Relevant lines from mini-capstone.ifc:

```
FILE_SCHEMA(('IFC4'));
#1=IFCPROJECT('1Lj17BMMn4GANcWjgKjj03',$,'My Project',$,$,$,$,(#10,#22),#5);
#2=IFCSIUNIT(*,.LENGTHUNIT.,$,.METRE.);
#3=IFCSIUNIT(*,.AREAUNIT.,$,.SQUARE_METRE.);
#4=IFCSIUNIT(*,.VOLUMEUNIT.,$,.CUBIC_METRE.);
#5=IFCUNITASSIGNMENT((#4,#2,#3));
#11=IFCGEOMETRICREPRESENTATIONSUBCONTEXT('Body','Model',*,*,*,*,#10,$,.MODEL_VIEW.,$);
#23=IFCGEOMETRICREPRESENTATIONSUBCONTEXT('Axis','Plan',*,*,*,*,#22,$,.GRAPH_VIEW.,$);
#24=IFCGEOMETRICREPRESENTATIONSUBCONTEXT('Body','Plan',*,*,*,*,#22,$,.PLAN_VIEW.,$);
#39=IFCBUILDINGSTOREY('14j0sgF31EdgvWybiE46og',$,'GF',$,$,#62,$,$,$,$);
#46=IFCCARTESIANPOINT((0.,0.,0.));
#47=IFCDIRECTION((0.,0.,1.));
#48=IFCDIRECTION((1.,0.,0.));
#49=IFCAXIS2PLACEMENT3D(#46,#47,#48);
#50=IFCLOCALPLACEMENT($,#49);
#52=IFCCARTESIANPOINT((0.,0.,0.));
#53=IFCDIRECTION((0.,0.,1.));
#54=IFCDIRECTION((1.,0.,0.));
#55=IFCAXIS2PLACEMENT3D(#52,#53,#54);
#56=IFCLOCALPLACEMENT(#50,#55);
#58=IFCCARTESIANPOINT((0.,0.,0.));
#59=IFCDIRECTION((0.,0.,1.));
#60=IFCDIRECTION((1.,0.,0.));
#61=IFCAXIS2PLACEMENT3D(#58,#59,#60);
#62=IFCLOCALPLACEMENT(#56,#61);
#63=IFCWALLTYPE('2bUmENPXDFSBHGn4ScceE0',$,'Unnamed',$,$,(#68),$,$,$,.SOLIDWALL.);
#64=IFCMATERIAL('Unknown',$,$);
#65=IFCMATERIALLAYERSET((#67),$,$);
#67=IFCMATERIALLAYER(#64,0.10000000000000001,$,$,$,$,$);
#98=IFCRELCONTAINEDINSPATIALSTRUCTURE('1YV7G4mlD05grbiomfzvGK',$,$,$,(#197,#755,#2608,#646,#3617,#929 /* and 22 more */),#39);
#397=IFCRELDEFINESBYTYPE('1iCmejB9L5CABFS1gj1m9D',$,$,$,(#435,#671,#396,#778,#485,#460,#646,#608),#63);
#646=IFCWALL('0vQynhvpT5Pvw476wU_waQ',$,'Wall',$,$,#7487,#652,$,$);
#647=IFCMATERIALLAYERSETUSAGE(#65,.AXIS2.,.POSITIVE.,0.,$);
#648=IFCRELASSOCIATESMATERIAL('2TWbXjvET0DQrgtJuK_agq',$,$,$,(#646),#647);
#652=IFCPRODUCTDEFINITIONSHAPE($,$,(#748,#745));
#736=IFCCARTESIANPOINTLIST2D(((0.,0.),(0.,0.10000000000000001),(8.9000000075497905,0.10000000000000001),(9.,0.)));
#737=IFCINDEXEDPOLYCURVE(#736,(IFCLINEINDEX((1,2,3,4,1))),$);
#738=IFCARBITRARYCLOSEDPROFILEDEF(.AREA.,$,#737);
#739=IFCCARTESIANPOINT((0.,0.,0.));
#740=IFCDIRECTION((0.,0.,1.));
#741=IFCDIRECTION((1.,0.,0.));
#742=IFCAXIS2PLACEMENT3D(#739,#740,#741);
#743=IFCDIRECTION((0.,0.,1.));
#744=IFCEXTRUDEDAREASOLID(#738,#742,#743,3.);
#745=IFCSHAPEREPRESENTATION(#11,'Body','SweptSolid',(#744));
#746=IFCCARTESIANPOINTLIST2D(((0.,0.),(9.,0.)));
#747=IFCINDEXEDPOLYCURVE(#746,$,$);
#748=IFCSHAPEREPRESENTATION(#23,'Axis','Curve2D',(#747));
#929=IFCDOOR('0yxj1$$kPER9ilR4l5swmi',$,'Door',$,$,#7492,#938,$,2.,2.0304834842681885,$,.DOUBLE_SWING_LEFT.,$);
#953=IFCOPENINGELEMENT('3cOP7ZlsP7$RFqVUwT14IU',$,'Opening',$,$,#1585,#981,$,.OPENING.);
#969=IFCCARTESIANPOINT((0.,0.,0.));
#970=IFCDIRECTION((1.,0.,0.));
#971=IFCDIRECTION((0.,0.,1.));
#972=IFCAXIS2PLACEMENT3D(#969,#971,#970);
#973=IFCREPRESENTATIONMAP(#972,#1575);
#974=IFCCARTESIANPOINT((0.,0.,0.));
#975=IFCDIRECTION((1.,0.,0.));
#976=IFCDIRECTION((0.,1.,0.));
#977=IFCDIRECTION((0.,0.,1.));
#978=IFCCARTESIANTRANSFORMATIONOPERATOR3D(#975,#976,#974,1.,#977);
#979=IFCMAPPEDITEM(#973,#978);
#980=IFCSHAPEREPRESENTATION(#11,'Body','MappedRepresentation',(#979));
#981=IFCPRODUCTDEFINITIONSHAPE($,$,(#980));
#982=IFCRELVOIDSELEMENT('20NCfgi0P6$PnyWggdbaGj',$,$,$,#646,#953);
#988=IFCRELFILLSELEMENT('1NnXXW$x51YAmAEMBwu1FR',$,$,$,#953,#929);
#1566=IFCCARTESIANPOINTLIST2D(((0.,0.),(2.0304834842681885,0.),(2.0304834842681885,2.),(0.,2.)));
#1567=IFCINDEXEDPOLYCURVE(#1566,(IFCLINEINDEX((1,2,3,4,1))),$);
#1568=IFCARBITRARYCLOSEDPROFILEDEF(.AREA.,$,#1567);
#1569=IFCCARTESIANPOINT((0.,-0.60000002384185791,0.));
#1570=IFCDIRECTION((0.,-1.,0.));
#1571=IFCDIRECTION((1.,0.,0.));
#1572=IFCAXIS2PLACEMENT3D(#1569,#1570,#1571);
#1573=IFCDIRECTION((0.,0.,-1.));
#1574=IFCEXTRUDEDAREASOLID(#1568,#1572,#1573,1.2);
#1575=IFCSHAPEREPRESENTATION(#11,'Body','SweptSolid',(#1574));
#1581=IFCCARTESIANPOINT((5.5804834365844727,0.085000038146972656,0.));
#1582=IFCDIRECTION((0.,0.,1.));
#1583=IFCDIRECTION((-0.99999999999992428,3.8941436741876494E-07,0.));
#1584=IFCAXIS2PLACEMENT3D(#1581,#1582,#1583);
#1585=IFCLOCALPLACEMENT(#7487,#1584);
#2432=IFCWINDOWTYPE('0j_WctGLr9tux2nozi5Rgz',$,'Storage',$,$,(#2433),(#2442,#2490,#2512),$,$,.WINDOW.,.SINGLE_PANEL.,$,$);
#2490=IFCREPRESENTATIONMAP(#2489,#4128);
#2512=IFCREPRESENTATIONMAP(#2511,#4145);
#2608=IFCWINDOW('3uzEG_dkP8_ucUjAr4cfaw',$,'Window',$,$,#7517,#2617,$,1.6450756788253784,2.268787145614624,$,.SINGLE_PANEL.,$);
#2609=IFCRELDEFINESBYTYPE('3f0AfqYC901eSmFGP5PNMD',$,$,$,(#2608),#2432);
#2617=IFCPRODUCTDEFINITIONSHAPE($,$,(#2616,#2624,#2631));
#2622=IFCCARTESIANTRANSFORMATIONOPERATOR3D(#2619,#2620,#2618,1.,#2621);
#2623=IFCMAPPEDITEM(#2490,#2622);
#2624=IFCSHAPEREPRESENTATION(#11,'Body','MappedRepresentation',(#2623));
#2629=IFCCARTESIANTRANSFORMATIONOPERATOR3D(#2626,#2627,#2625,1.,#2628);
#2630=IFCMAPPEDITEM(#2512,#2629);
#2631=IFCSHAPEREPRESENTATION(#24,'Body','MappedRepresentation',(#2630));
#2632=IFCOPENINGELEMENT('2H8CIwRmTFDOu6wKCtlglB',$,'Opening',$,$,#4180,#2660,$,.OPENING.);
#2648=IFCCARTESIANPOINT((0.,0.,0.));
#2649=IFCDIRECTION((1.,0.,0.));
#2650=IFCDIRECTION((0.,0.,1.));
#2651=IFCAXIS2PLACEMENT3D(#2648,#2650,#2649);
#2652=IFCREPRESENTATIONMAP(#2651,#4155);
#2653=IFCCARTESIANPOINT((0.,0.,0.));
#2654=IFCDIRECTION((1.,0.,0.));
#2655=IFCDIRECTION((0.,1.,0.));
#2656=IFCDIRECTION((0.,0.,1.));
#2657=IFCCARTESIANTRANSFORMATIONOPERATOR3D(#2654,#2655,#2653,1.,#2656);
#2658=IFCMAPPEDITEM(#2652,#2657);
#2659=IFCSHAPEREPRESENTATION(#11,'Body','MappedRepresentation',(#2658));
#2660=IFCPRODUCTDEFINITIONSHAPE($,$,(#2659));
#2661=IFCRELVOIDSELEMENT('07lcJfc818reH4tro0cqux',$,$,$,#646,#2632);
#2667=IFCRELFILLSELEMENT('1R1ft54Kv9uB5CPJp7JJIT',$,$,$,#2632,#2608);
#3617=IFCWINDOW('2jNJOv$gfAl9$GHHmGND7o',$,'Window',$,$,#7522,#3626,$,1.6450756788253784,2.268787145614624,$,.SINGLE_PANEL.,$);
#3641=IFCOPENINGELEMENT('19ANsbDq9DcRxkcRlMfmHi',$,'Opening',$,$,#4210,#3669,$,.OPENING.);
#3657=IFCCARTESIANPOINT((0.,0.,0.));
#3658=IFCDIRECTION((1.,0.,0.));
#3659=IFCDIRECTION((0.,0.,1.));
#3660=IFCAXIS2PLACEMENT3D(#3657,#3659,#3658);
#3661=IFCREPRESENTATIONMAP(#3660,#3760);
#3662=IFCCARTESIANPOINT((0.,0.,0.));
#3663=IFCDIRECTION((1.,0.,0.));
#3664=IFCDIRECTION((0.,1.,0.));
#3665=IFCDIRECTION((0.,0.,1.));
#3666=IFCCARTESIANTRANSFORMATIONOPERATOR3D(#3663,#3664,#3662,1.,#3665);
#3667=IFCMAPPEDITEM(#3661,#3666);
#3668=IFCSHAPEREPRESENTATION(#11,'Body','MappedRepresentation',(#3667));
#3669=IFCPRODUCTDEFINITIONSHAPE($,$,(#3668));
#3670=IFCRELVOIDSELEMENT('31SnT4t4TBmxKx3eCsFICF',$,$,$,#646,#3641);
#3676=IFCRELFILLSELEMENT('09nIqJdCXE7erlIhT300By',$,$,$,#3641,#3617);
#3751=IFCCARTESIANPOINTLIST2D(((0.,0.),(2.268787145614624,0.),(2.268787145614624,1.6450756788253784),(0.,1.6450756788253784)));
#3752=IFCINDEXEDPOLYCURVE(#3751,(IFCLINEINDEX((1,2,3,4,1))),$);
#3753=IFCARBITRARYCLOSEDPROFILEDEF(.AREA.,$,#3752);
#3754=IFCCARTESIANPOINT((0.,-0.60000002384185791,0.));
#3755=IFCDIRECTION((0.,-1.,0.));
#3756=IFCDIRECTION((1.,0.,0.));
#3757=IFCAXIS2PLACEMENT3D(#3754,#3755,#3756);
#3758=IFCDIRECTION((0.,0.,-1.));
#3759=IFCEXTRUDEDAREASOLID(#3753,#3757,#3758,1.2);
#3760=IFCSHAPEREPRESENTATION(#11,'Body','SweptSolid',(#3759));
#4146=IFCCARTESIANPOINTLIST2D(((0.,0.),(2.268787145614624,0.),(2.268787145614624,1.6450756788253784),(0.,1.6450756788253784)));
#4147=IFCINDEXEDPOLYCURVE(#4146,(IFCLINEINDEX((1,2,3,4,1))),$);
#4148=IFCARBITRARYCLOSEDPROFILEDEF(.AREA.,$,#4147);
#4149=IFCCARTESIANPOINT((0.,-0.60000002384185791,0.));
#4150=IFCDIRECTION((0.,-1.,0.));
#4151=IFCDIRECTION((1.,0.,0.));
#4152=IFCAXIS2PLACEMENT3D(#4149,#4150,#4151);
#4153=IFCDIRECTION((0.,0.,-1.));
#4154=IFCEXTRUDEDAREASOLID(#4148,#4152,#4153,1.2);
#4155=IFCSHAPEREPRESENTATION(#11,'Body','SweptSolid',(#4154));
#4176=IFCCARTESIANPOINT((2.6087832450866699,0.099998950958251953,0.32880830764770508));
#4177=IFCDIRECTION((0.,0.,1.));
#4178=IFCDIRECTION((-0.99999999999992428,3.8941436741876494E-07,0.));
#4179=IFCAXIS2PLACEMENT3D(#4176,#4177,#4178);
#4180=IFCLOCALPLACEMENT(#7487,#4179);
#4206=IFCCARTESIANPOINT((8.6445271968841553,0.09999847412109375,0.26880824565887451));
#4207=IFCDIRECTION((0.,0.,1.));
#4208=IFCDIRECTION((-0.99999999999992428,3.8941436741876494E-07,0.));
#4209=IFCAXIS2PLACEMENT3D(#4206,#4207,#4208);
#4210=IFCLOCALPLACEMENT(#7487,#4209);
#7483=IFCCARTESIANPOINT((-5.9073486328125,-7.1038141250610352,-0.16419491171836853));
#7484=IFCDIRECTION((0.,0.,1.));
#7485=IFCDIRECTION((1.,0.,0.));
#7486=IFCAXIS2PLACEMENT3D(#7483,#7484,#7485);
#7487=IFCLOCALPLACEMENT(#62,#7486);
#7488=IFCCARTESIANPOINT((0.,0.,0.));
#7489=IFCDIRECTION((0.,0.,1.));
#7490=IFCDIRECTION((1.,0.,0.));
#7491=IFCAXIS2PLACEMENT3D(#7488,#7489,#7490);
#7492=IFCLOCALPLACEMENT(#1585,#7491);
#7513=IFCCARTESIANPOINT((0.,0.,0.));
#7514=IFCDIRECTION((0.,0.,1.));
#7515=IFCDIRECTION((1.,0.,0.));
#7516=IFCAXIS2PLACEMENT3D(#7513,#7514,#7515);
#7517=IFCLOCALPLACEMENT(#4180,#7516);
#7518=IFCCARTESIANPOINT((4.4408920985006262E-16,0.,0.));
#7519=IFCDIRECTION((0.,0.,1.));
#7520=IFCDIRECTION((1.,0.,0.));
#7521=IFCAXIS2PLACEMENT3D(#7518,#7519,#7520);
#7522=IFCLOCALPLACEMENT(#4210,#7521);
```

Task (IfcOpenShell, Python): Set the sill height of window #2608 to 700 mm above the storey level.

```python
import numpy as np
import ifcopenshell
import ifcopenshell.api.geometry
import ifcopenshell.geom
import ifcopenshell.util.element
import ifcopenshell.util.placement
import ifcopenshell.util.shape
import ifcopenshell.util.unit

model = ifcopenshell.open("mini-capstone.ifc")
unit_scale = ifcopenshell.util.unit.calculate_unit_scale(model)

window = model.by_guid("3uzEG_dkP8_ucUjAr4cfaw")
opening = window.FillsVoids[0].RelatingOpeningElement
storey = ifcopenshell.util.element.get_container(window, ifc_class="IfcBuildingStorey")
level = ifcopenshell.util.placement.get_local_placement(storey.ObjectPlacement)[2, 3]

# The opening's origin need not be at the sill, so measure its lowest point.
shape = ifcopenshell.geom.create_shape(ifcopenshell.geom.settings(), opening)
bottom = ifcopenshell.util.shape.get_shape_bottom_elevation(shape, shape.geometry) / unit_scale
dz = level + 0.7 - bottom

shift = np.array([0.0, 0.0, dz])
# The window is placed relative to its opening, so it follows when the opening moves.
matrix = ifcopenshell.util.placement.get_local_placement(opening.ObjectPlacement)
matrix[:3, 3] += shift
ifcopenshell.api.geometry.edit_object_placement(
    model, product=opening, matrix=matrix, is_si=False, should_transform_children=True
)

print(f"moved by {dz * unit_scale:+.3f} m")

model.write("mini-capstone_rev.ifc")
```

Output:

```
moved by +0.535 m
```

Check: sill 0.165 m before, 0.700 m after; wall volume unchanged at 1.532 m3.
